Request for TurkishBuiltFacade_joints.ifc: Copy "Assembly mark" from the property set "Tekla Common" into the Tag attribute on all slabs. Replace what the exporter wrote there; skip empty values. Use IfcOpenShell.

First a look at what the model holds.

```python
import ifcopenshell
import ifcopenshell.util.element

model = ifcopenshell.open("TurkishBuiltFacade_joints.ifc")
print(model.schema)
slabs = model.by_type("IfcSlab")
print(len(slabs), "slabs")
for e in slabs[:8]:
    source = ifcopenshell.util.element.get_pset(e, "Tekla Common", "Assembly mark")
    target = e.Tag
    print(e.id(), repr(source), repr(target), sep=" | ")
```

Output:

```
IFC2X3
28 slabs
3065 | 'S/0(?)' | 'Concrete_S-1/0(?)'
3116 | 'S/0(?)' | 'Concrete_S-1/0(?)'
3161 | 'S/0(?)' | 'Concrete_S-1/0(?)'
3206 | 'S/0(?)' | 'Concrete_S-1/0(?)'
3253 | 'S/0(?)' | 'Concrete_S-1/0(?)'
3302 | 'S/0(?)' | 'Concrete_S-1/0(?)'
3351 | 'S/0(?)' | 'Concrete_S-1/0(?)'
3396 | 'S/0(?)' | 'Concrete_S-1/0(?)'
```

```python
import ifcopenshell
import ifcopenshell.util.element

model = ifcopenshell.open("TurkishBuiltFacade_joints.ifc")

count = 0
for e in model.by_type("IfcSlab"):
    value = ifcopenshell.util.element.get_pset(e, "Tekla Common", "Assembly mark")
    current = e.Tag
    if not value or not value.strip() or current == value:
        continue
    e.Tag = value
    count += 1

print(count, "slabs updated")

model.write("TurkishBuiltFacade_joints_v2.ifc")
```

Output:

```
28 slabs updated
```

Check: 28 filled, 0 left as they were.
